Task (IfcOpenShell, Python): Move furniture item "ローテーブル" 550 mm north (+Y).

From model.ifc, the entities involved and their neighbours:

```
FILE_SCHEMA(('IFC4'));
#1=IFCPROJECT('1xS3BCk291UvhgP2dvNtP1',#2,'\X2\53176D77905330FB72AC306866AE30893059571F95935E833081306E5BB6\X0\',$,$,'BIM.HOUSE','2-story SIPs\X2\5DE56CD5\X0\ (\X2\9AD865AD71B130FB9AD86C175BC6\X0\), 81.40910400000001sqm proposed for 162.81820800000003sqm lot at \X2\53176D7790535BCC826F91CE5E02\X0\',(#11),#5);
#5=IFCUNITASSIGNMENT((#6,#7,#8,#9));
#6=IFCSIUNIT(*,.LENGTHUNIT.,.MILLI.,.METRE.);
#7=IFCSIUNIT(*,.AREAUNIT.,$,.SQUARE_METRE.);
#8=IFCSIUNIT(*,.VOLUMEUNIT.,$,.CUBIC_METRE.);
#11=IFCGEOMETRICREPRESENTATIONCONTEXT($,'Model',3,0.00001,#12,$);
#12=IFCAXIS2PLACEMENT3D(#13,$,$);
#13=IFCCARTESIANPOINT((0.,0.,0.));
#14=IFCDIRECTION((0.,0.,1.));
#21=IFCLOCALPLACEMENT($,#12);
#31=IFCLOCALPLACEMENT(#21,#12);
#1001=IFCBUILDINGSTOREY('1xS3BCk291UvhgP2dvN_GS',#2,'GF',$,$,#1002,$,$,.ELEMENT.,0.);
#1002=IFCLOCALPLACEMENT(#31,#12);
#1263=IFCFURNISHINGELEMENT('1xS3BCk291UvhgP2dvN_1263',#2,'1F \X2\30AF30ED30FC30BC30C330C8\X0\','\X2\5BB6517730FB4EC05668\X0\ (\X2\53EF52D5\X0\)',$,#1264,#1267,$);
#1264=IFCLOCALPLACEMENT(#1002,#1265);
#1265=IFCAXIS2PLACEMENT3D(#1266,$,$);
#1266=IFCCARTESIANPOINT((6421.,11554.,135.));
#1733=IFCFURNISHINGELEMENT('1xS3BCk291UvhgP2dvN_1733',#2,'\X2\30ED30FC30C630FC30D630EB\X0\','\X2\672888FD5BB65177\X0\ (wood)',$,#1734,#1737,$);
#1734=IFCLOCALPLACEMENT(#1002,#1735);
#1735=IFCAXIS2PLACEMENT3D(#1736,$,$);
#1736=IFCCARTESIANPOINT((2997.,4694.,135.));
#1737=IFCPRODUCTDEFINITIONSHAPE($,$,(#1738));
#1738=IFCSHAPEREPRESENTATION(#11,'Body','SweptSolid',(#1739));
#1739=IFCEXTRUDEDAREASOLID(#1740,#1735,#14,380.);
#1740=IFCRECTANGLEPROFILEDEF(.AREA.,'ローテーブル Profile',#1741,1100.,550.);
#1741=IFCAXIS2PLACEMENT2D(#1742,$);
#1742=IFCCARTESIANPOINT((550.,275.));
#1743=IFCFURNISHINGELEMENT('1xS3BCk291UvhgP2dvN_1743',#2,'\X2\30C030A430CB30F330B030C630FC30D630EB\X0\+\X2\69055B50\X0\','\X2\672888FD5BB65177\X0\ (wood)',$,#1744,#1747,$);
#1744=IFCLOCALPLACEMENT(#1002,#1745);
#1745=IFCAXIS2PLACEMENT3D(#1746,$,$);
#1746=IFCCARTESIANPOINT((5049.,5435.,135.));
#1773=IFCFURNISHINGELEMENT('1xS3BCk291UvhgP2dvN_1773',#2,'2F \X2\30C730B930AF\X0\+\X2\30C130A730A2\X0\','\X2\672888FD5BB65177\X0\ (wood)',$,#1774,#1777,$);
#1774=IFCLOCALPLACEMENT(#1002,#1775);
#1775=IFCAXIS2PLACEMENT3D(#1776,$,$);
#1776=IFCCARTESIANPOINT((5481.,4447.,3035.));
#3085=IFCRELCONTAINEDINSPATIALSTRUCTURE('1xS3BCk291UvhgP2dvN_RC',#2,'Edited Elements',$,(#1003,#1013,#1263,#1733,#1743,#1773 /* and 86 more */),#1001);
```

```python
import ifcopenshell
import ifcopenshell.api.geometry
import ifcopenshell.util.placement

model = ifcopenshell.open("model.ifc")

item = model.by_guid("1xS3BCk291UvhgP2dvN_1733")
matrix = ifcopenshell.util.placement.get_local_placement(item.ObjectPlacement)
matrix[1, 3] += 550.0
ifcopenshell.api.geometry.edit_object_placement(model, product=item, matrix=matrix, is_si=False)

print(ifcopenshell.util.placement.get_local_placement(item.ObjectPlacement).round(3) + 0.0)

model.write("model_updated.ifc")
```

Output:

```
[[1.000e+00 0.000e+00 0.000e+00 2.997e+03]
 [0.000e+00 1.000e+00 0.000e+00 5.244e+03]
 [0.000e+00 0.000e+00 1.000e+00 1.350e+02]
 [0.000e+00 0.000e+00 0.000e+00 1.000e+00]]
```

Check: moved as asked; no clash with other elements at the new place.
